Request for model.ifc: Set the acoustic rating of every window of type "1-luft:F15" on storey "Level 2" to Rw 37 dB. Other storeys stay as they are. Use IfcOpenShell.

First a look at what the model holds.

```python
import ifcopenshell
import ifcopenshell.util.element

model = ifcopenshell.open("model.ifc")
print(model.schema)
storey = next(s for s in model.by_type("IfcBuildingStorey") if s.Name == "Level 2")
windows = [e for e in ifcopenshell.util.element.get_decomposition(storey) if e.is_a("IfcWindow")]
seen = {}
for e in windows:
    element_type = ifcopenshell.util.element.get_type(e)
    key = (element_type.Name if element_type != e and element_type else None, ifcopenshell.util.element.get_pset(e, "Pset_WindowCommon", "AcousticRating"))
    seen[key] = seen.get(key, 0) + 1
for (name, value), count in sorted(seen.items(), key=str):
    print(count, "x", name, "|", value)
```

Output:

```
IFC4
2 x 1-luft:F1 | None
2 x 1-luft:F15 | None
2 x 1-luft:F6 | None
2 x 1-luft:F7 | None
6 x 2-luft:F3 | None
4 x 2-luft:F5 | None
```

```python
import ifcopenshell
import ifcopenshell.api.pset
import ifcopenshell.util.element

model = ifcopenshell.open("model.ifc")

storey = next(s for s in model.by_type("IfcBuildingStorey") if s.Name == "Level 2")
windows = [e for e in ifcopenshell.util.element.get_decomposition(storey) if e.is_a("IfcWindow")]

count = 0
for e in windows:
    element_type = ifcopenshell.util.element.get_type(e)
    if element_type in (None, e) or element_type.Name != "1-luft:F15":
        continue
    # add_pset returns the element's existing set when there is one.
    pset = ifcopenshell.api.pset.add_pset(model, product=e, name="Pset_WindowCommon")
    ifcopenshell.api.pset.edit_pset(model, pset=pset, properties={"AcousticRating": "Rw 37 dB"})
    count += 1

print(count, "windows updated")

model.write("model_rev.ifc")
```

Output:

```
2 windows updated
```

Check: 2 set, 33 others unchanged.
